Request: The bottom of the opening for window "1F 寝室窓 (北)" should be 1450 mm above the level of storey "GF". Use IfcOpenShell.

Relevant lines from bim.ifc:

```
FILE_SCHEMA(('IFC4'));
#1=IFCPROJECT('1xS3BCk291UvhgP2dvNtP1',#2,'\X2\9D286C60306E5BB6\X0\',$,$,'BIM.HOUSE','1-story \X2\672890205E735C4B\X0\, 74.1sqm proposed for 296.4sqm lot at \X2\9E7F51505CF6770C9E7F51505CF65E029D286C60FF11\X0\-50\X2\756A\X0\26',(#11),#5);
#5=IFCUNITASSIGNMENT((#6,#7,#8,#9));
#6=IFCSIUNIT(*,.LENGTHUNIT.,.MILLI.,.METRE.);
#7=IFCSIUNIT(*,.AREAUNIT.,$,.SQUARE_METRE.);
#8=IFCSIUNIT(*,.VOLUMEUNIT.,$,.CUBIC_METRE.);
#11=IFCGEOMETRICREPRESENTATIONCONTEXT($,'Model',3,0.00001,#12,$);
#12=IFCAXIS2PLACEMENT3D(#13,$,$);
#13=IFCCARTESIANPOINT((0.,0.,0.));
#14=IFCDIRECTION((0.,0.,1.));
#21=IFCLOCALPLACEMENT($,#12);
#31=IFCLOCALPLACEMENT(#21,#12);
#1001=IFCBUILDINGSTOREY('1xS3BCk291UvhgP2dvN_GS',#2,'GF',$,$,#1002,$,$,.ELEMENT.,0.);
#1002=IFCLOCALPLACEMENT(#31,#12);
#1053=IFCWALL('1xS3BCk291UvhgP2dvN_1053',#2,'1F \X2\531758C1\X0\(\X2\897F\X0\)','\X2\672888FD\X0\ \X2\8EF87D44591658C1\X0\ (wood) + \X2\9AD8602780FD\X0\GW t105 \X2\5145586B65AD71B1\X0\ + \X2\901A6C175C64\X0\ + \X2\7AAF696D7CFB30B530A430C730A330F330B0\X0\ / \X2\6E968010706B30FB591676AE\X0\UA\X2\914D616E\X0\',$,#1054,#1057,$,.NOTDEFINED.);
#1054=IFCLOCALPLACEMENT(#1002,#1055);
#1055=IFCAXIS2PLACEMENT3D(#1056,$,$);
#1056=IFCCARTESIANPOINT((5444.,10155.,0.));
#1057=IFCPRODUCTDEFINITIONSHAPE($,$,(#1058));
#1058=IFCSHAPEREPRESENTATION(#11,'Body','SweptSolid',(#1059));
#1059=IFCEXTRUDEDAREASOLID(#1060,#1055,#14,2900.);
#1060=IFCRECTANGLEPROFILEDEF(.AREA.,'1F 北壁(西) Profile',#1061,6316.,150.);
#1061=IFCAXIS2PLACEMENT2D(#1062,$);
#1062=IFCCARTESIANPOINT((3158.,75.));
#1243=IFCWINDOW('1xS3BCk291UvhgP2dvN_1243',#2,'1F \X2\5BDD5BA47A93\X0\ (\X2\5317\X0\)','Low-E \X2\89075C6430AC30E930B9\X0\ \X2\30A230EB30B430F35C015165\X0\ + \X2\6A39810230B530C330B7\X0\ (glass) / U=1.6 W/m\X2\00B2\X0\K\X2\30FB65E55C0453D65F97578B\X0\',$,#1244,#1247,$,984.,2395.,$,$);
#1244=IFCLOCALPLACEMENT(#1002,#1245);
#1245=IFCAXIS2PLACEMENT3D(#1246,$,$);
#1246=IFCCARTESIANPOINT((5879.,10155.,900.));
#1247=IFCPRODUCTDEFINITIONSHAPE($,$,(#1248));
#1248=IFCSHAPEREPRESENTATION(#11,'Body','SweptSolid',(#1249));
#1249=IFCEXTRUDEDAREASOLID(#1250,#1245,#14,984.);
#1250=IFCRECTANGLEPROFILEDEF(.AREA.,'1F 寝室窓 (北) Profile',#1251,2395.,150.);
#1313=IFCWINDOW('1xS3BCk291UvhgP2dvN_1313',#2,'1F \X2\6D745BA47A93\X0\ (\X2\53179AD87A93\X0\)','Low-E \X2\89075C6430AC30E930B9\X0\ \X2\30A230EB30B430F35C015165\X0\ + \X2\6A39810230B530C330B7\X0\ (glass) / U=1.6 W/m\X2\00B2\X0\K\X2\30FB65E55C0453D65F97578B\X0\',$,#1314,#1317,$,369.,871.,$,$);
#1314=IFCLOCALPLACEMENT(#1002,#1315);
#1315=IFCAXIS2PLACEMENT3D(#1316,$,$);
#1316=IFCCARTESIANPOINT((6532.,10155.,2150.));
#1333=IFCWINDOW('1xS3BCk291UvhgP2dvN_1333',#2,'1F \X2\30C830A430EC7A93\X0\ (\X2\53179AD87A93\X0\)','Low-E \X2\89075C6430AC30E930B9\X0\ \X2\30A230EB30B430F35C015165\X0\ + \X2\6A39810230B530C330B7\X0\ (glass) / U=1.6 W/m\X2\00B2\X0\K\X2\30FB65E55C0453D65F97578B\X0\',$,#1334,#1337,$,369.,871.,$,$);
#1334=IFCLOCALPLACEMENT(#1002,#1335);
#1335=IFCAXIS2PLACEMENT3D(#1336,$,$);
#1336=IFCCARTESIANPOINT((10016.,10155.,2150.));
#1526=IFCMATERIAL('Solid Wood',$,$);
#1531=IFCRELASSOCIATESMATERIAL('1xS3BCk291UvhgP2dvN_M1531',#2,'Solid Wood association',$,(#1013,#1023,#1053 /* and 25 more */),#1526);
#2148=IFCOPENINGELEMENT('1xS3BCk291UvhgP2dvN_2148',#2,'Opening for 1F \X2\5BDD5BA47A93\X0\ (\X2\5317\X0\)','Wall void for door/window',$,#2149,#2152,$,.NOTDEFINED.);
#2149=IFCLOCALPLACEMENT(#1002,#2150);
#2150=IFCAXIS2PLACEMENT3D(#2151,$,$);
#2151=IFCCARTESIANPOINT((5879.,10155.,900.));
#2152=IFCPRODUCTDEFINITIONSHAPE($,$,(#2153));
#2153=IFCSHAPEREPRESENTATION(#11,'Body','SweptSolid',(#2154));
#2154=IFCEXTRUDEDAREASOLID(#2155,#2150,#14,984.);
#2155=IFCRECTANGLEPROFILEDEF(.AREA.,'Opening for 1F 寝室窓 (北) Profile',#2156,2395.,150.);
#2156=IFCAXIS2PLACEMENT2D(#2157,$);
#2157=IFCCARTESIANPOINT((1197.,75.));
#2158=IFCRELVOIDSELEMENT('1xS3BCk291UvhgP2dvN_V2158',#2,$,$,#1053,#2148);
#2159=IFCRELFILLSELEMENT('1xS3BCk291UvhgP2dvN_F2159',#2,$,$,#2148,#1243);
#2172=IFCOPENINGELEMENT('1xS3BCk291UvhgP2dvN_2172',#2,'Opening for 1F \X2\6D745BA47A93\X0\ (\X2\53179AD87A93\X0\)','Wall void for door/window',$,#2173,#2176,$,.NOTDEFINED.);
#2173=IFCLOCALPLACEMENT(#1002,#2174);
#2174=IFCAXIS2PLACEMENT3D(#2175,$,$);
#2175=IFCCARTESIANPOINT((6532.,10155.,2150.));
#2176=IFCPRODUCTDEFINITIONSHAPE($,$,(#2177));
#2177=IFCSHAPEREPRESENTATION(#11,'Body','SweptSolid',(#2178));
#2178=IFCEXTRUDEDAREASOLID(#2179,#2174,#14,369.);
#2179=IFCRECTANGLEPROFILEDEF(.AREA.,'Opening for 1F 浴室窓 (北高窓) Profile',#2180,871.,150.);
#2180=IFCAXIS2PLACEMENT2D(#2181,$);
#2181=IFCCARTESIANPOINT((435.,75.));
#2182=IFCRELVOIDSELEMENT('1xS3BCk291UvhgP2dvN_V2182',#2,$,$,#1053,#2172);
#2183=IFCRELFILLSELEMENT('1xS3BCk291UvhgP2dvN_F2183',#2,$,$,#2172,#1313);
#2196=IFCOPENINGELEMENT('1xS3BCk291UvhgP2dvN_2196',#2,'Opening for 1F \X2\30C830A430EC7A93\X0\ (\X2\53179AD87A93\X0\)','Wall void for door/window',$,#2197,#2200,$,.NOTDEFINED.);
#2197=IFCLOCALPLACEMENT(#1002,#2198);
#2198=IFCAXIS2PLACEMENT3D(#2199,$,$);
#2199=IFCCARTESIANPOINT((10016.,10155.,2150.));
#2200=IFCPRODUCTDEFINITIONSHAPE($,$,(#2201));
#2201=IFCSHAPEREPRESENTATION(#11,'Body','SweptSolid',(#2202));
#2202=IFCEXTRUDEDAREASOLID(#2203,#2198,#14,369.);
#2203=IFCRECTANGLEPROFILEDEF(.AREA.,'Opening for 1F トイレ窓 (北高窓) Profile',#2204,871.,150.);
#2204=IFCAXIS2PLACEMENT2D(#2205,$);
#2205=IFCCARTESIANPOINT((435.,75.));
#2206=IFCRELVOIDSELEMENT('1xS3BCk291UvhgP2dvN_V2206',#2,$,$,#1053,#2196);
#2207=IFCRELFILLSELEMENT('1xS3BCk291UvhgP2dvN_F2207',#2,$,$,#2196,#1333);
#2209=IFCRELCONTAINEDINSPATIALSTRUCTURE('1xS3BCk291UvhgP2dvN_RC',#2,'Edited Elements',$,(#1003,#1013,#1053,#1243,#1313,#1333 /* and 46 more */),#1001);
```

```python
import numpy as np
import ifcopenshell
import ifcopenshell.api.geometry
import ifcopenshell.geom
import ifcopenshell.util.element
import ifcopenshell.util.placement
import ifcopenshell.util.shape
import ifcopenshell.util.unit

model = ifcopenshell.open("bim.ifc")
unit_scale = ifcopenshell.util.unit.calculate_unit_scale(model)

window = model.by_guid("1xS3BCk291UvhgP2dvN_1243")
opening = window.FillsVoids[0].RelatingOpeningElement
storey = ifcopenshell.util.element.get_container(window, ifc_class="IfcBuildingStorey")
level = ifcopenshell.util.placement.get_local_placement(storey.ObjectPlacement)[2, 3]

# The opening's origin need not be at the sill, so measure its lowest point.
shape = ifcopenshell.geom.create_shape(ifcopenshell.geom.settings(), opening)
bottom = ifcopenshell.util.shape.get_shape_bottom_elevation(shape, shape.geometry) / unit_scale
dz = level + 1450.0 - bottom

shift = np.array([0.0, 0.0, dz])
# The window is not placed relative to its opening, so move both.
for product in (opening, window):
    matrix = ifcopenshell.util.placement.get_local_placement(product.ObjectPlacement)
    matrix[:3, 3] += shift
    ifcopenshell.api.geometry.edit_object_placement(model, product=product, matrix=matrix, is_si=False)

print(f"moved by {dz * unit_scale:+.3f} m")

model.write("bim-out.ifc")
```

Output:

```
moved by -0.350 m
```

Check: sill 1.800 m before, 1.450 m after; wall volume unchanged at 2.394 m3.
